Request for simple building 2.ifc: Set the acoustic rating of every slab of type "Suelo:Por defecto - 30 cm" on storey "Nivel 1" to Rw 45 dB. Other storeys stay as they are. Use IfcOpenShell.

First a look at what the model holds.

```python
import ifcopenshell
import ifcopenshell.util.element

model = ifcopenshell.open("simple building 2.ifc")
print(model.schema)
storey = next(s for s in model.by_type("IfcBuildingStorey") if s.Name == "Nivel 1")
slabs = [e for e in ifcopenshell.util.element.get_decomposition(storey) if e.is_a("IfcSlab")]
seen = {}
for e in slabs:
    element_type = ifcopenshell.util.element.get_type(e)
    key = (element_type.Name if element_type != e and element_type else None, ifcopenshell.util.element.get_pset(e, "Pset_SlabCommon", "AcousticRating"))
    seen[key] = seen.get(key, 0) + 1
for (name, value), count in sorted(seen.items(), key=str):
    print(count, "x", name, "|", value)
```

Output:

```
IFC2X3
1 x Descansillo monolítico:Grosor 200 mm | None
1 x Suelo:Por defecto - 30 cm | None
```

```python
import ifcopenshell
import ifcopenshell.api.pset
import ifcopenshell.util.element

model = ifcopenshell.open("simple building 2.ifc")

storey = next(s for s in model.by_type("IfcBuildingStorey") if s.Name == "Nivel 1")
slabs = [e for e in ifcopenshell.util.element.get_decomposition(storey) if e.is_a("IfcSlab")]

count = 0
for e in slabs:
    element_type = ifcopenshell.util.element.get_type(e)
    if element_type in (None, e) or element_type.Name != "Suelo:Por defecto - 30 cm":
        continue
    # add_pset returns the element's existing set when there is one.
    pset = ifcopenshell.api.pset.add_pset(model, product=e, name="Pset_SlabCommon")
    ifcopenshell.api.pset.edit_pset(model, pset=pset, properties={"AcousticRating": "Rw 45 dB"})
    count += 1

print(count, "slabs updated")

model.write("simple building 2-out.ifc")
```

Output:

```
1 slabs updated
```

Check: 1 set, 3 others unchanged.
